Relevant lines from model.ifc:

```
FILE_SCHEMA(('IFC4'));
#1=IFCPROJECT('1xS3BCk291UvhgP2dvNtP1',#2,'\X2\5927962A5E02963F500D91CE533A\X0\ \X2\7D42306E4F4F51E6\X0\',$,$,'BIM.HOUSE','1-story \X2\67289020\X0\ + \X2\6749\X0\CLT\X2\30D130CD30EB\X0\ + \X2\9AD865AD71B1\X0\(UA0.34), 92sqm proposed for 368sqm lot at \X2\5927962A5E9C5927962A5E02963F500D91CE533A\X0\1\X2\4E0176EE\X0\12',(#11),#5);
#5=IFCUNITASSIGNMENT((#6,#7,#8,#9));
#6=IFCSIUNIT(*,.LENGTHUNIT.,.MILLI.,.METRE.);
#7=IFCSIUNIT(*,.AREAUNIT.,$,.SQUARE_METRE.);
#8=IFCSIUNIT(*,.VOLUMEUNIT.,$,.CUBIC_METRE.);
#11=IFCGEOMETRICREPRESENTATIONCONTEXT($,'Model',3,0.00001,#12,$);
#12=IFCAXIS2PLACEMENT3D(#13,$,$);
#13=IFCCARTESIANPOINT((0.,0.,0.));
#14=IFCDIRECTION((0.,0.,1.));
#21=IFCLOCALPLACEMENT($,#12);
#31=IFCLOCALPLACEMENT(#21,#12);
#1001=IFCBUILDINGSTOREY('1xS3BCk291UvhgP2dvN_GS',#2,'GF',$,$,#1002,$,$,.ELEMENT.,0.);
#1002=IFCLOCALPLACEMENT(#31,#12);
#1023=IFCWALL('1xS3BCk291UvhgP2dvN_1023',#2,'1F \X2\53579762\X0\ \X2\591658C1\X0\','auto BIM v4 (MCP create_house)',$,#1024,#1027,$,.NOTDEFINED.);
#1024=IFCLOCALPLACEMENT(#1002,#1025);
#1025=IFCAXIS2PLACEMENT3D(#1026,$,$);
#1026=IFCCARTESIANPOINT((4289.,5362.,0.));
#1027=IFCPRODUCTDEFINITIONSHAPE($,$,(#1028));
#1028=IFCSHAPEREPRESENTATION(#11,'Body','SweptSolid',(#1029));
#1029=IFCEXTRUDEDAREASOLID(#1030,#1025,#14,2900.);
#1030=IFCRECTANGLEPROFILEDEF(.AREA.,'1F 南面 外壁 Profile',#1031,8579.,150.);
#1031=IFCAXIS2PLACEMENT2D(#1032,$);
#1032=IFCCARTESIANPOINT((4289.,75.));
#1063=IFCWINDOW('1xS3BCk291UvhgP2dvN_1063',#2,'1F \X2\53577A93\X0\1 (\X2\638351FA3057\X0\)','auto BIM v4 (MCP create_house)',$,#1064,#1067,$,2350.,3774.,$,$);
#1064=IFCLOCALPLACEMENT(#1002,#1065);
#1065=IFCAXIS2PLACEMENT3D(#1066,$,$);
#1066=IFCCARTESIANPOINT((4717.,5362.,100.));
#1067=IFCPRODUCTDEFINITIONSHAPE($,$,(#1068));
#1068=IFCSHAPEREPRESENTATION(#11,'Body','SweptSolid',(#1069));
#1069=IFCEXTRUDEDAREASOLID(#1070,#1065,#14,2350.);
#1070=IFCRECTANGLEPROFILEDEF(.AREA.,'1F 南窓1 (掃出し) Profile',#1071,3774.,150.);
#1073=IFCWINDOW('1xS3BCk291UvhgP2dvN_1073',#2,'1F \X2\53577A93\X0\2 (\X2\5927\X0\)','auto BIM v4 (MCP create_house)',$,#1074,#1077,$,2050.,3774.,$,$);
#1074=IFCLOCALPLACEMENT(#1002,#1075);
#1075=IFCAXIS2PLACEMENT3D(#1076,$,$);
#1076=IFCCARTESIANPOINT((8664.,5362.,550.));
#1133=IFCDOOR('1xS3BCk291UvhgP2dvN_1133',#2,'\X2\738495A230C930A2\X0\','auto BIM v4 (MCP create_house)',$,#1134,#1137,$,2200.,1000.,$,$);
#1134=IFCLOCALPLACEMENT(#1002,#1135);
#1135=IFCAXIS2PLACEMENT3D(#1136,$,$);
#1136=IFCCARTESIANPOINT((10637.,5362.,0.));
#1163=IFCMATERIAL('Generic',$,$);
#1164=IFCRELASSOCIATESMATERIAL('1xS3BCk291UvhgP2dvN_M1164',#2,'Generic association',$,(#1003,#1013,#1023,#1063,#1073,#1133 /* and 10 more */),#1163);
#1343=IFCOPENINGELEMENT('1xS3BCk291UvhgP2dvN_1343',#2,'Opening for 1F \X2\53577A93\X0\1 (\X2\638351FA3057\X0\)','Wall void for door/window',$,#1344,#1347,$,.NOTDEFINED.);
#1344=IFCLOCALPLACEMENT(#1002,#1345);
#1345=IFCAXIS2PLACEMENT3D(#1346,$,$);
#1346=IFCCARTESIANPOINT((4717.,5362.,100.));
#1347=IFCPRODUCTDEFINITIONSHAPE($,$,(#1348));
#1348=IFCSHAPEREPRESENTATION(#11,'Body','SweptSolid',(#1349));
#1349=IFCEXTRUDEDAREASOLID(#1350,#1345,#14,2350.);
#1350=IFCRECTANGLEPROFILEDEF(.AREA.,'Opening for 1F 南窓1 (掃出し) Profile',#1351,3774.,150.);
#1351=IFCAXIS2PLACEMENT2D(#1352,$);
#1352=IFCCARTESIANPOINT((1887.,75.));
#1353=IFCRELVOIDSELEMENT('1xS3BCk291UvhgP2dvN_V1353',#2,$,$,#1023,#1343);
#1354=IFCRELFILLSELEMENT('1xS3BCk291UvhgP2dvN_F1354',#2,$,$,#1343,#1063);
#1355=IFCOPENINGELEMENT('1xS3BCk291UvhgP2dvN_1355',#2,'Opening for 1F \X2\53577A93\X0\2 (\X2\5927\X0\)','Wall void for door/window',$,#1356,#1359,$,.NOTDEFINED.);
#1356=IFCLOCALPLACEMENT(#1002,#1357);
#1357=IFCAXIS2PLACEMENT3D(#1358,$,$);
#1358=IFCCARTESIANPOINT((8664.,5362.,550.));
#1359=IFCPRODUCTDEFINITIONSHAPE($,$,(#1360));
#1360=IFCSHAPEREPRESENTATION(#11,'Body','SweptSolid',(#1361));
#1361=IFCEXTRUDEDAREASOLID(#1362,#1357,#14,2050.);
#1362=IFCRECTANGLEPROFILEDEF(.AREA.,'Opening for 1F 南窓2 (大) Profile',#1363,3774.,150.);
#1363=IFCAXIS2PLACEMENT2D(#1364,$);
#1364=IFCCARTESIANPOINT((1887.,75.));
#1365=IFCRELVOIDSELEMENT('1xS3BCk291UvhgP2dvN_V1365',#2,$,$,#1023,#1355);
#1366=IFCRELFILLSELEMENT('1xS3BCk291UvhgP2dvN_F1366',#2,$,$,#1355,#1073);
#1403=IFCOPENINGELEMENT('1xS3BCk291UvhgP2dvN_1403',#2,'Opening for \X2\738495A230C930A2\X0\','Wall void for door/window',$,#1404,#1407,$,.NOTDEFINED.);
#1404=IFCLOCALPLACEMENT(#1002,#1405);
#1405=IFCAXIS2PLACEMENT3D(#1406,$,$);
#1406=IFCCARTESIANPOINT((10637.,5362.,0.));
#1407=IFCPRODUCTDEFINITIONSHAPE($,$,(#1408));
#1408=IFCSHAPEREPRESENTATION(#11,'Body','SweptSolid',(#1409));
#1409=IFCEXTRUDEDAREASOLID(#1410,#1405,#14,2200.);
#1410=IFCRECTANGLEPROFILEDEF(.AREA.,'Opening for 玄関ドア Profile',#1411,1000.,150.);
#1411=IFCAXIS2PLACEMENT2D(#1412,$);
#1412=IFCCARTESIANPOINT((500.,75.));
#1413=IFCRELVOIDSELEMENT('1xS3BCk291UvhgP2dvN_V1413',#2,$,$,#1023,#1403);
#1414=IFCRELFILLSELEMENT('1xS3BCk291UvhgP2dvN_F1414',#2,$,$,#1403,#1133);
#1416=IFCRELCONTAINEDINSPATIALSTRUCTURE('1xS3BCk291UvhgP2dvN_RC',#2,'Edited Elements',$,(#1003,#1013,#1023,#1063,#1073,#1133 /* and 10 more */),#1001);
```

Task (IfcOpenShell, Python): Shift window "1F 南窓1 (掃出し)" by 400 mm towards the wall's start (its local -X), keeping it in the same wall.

```python
import ifcopenshell
import ifcopenshell.api.geometry
import ifcopenshell.util.placement
import ifcopenshell.util.unit

model = ifcopenshell.open("model.ifc")
unit_scale = ifcopenshell.util.unit.calculate_unit_scale(model)

window = model.by_guid("1xS3BCk291UvhgP2dvN_1063")
opening = window.FillsVoids[0].RelatingOpeningElement
wall = opening.VoidsElements[0].RelatingBuildingElement

wall_matrix = ifcopenshell.util.placement.get_local_placement(wall.ObjectPlacement)
shift = wall_matrix[:3, 0] * -0.4 / unit_scale
before = ifcopenshell.util.placement.get_local_placement(window.ObjectPlacement)[:3, 3].copy()

# The window is not placed relative to its opening, so move both.
for product in (opening, window):
    matrix = ifcopenshell.util.placement.get_local_placement(product.ObjectPlacement)
    matrix[:3, 3] += shift
    ifcopenshell.api.geometry.edit_object_placement(model, product=product, matrix=matrix, is_si=False)

after = ifcopenshell.util.placement.get_local_placement(window.ObjectPlacement)[:3, 3]
print("window moved by", (after - before).round(3) + 0.0)

model.write("model-out.ifc")
```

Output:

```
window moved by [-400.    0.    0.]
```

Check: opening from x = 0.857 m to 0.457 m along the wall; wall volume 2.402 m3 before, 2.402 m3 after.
